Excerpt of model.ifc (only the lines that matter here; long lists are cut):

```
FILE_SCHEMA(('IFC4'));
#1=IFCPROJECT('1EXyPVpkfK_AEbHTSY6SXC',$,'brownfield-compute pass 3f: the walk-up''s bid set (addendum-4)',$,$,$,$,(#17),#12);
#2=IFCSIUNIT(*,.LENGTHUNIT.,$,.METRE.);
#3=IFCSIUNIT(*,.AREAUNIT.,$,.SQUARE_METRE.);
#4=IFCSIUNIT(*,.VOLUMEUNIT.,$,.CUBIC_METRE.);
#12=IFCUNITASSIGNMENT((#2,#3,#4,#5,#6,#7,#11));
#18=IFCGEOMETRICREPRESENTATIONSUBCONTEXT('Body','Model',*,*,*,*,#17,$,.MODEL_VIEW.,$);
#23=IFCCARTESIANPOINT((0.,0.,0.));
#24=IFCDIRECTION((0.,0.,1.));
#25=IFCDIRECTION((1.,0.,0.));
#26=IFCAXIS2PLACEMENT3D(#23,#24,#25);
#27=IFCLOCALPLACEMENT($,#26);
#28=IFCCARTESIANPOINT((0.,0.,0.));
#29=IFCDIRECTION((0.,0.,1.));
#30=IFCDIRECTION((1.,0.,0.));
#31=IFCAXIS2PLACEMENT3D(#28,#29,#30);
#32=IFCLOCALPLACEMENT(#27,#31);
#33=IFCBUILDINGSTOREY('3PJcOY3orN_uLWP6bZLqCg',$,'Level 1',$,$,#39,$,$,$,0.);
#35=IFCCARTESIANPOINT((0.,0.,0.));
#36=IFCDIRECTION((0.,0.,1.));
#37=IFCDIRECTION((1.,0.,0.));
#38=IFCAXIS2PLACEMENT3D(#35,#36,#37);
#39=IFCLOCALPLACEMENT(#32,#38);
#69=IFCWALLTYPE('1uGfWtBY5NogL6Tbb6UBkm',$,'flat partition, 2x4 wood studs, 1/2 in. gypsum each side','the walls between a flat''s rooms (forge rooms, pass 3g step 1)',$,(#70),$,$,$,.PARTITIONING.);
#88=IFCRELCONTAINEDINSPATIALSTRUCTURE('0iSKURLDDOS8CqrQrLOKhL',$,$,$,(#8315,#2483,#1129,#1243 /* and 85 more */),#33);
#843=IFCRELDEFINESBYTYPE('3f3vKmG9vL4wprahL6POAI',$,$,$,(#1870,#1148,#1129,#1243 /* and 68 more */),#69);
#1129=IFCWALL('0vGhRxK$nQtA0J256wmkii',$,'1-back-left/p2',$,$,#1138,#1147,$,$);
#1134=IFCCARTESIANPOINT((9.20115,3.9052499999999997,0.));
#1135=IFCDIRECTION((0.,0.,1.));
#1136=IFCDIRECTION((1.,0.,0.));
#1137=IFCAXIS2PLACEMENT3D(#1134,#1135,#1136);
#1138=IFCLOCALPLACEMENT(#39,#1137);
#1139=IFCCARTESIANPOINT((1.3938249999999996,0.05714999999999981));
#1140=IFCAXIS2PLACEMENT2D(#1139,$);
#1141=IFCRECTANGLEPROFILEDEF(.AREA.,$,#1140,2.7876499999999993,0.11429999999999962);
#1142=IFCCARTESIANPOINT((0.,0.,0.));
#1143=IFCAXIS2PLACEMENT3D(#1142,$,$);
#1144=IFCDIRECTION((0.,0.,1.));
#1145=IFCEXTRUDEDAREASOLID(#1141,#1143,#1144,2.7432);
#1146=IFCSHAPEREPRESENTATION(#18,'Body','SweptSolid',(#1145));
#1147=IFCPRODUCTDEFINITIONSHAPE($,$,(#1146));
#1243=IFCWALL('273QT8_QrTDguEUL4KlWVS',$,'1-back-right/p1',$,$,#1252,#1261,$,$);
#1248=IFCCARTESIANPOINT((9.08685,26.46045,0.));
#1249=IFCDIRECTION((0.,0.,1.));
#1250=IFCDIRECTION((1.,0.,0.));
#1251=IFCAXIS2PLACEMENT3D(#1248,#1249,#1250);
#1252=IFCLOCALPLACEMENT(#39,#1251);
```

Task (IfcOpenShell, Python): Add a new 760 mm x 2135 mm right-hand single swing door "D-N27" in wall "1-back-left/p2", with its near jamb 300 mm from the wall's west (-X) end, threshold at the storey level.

```python
import numpy as np
import ifcopenshell
import ifcopenshell.api.feature
import ifcopenshell.api.geometry
import ifcopenshell.api.root
import ifcopenshell.api.spatial
import ifcopenshell.geom
import ifcopenshell.util.element
import ifcopenshell.util.placement
import ifcopenshell.util.representation
import ifcopenshell.util.shape
import ifcopenshell.util.unit

model = ifcopenshell.open("model.ifc")
unit_scale = ifcopenshell.util.unit.calculate_unit_scale(model)
settings = ifcopenshell.geom.settings()


def volume(element):
    """Net volume in cubic metres, openings subtracted."""
    shape = ifcopenshell.geom.create_shape(settings, element)
    return ifcopenshell.util.shape.get_volume(shape.geometry)


wall = model.by_id(1129)
storey = ifcopenshell.util.element.get_container(wall, ifc_class="IfcBuildingStorey")
context = ifcopenshell.util.representation.get_context(model, "Model", "Body", "MODEL_VIEW")
before = volume(wall)

width, height, from_end, sill = 0.76, 2.135, 0.3, 0.0  # metres

# The wall runs along its own X axis, and the end named is its -X end.
wall_shape = ifcopenshell.geom.create_shape(settings, wall)
x, y, z = ifcopenshell.util.shape.get_vertices(wall_shape.geometry).T
start = x.min() + from_end
face, thickness = float(y.min()), float(y.max() - y.min())
wall_matrix = ifcopenshell.util.placement.get_local_placement(wall.ObjectPlacement)
level = ifcopenshell.util.placement.get_local_placement(storey.ObjectPlacement)[2, 3]


def in_wall(x, y):
    """Placement at x, y metres in the wall's axes, at sill height."""
    matrix = wall_matrix.copy()
    matrix[:, 3] = wall_matrix @ np.array([x / unit_scale, y / unit_scale, 0.0, 1.0])
    matrix[2, 3] = level + sill / unit_scale
    return matrix


# Opening: a box that overshoots both wall faces by 50 mm.
opening = ifcopenshell.api.root.create_entity(model, ifc_class="IfcOpeningElement", predefined_type="OPENING")
box = ifcopenshell.api.geometry.add_wall_representation(
    model, context=context, length=width, height=height, thickness=thickness + 0.1
)
ifcopenshell.api.geometry.assign_representation(model, product=opening, representation=box)
ifcopenshell.api.geometry.edit_object_placement(model, product=opening, matrix=in_wall(start, face - 0.05), is_si=False)
ifcopenshell.api.feature.add_feature(model, feature=opening, element=wall)

door = ifcopenshell.api.root.create_entity(model, ifc_class="IfcDoor", name="D-N27", predefined_type="DOOR")
door.OverallWidth, door.OverallHeight = width / unit_scale, height / unit_scale
door.OperationType = "SINGLE_SWING_RIGHT"
body = ifcopenshell.api.geometry.add_door_representation(
    model,
    context=context,
    overall_width=door.OverallWidth,
    overall_height=door.OverallHeight,
    operation_type="SINGLE_SWING_RIGHT",
    lining_properties={"LiningDepth": thickness / unit_scale, "ThresholdDepth": thickness / unit_scale},
)
ifcopenshell.api.geometry.assign_representation(model, product=door, representation=body)
ifcopenshell.api.spatial.assign_container(model, products=[door], relating_structure=storey)
ifcopenshell.api.feature.add_filling(model, opening=opening, element=door)

# The lining spans the wall, so the door starts at the wall face.
ifcopenshell.api.geometry.edit_object_placement(model, product=door, matrix=in_wall(start, face), is_si=False)

after = volume(wall)

print(f"wall volume {before:.3f} -> {after:.3f} m3")

model.write("model_updated.ifc")
```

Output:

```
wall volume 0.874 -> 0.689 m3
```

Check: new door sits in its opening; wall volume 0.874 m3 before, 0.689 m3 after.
